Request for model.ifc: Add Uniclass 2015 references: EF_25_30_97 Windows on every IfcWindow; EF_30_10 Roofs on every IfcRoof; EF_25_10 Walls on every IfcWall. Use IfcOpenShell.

First a look at what the model holds.

```python
import ifcopenshell

model = ifcopenshell.open("model.ifc")
print(model.schema)
print("classifications:", [c.Name for c in model.by_type("IfcClassification")])
for ifc_class in ("IfcDoor", "IfcRoof", "IfcStair", "IfcWall", "IfcWindow"):
    print(ifc_class, len(model.by_type(ifc_class)))
```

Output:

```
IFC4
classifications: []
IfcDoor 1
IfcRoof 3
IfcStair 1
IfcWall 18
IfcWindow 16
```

```python
import ifcopenshell
import ifcopenshell.api.classification

model = ifcopenshell.open("model.ifc")

system = ifcopenshell.api.classification.add_classification(model, classification="Uniclass 2015")

codes = {
    "IfcWindow": ("EF_25_30_97", "Windows"),
    "IfcRoof": ("EF_30_10", "Roofs"),
    "IfcWall": ("EF_25_10", "Walls"),
}
for ifc_class, (code, name) in codes.items():
    products = model.by_type(ifc_class)
    ifcopenshell.api.classification.add_reference(
        model, products=products, classification=system, identification=code, name=name
    )
    print(code, len(products))

model.write("model_edited.ifc")
```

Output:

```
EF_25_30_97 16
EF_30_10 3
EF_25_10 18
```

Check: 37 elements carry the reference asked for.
